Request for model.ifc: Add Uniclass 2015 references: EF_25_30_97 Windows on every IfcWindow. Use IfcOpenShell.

First a look at what the model holds.

```python
import ifcopenshell

model = ifcopenshell.open("model.ifc")
print(model.schema)
print("classifications:", [c.Name for c in model.by_type("IfcClassification")])
for ifc_class in ("IfcDoor", "IfcRoof", "IfcStair", "IfcWall", "IfcWindow"):
    print(ifc_class, len(model.by_type(ifc_class)))
```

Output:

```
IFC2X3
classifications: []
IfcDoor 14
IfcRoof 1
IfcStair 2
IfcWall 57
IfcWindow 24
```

```python
import ifcopenshell
import ifcopenshell.api.classification

model = ifcopenshell.open("model.ifc")

# IFC2X3 requires Source and Edition and has no link from the project to the system.
system = model.create_entity("IfcClassification", Source="NBS", Edition="2015", Name="Uniclass 2015")

codes = {
    "IfcWindow": ("EF_25_30_97", "Windows"),
}
for ifc_class, (code, name) in codes.items():
    products = model.by_type(ifc_class)
    ifcopenshell.api.classification.add_reference(
        model, products=products, classification=system, identification=code, name=name
    )
    print(code, len(products))

model.write("model-out.ifc")
```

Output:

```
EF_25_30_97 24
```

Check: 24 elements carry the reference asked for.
